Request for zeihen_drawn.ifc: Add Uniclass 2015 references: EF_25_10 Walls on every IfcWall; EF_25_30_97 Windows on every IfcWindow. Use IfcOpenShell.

First a look at what the model holds.

```python
import ifcopenshell

model = ifcopenshell.open("zeihen_drawn.ifc")
print(model.schema)
print("classifications:", [c.Name for c in model.by_type("IfcClassification")])
for ifc_class in ("IfcDoor", "IfcRoof", "IfcStair", "IfcWall", "IfcWindow"):
    print(ifc_class, len(model.by_type(ifc_class)))
```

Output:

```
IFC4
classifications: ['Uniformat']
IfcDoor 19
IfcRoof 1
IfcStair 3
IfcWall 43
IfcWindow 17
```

```python
import ifcopenshell
import ifcopenshell.api.classification

model = ifcopenshell.open("zeihen_drawn.ifc")

system = ifcopenshell.api.classification.add_classification(model, classification="Uniclass 2015")

codes = {
    "IfcWall": ("EF_25_10", "Walls"),
    "IfcWindow": ("EF_25_30_97", "Windows"),
}
for ifc_class, (code, name) in codes.items():
    products = model.by_type(ifc_class)
    ifcopenshell.api.classification.add_reference(
        model, products=products, classification=system, identification=code, name=name
    )
    print(code, len(products))

model.write("zeihen_drawn_edited.ifc")
```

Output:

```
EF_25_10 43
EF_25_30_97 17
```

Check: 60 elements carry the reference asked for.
